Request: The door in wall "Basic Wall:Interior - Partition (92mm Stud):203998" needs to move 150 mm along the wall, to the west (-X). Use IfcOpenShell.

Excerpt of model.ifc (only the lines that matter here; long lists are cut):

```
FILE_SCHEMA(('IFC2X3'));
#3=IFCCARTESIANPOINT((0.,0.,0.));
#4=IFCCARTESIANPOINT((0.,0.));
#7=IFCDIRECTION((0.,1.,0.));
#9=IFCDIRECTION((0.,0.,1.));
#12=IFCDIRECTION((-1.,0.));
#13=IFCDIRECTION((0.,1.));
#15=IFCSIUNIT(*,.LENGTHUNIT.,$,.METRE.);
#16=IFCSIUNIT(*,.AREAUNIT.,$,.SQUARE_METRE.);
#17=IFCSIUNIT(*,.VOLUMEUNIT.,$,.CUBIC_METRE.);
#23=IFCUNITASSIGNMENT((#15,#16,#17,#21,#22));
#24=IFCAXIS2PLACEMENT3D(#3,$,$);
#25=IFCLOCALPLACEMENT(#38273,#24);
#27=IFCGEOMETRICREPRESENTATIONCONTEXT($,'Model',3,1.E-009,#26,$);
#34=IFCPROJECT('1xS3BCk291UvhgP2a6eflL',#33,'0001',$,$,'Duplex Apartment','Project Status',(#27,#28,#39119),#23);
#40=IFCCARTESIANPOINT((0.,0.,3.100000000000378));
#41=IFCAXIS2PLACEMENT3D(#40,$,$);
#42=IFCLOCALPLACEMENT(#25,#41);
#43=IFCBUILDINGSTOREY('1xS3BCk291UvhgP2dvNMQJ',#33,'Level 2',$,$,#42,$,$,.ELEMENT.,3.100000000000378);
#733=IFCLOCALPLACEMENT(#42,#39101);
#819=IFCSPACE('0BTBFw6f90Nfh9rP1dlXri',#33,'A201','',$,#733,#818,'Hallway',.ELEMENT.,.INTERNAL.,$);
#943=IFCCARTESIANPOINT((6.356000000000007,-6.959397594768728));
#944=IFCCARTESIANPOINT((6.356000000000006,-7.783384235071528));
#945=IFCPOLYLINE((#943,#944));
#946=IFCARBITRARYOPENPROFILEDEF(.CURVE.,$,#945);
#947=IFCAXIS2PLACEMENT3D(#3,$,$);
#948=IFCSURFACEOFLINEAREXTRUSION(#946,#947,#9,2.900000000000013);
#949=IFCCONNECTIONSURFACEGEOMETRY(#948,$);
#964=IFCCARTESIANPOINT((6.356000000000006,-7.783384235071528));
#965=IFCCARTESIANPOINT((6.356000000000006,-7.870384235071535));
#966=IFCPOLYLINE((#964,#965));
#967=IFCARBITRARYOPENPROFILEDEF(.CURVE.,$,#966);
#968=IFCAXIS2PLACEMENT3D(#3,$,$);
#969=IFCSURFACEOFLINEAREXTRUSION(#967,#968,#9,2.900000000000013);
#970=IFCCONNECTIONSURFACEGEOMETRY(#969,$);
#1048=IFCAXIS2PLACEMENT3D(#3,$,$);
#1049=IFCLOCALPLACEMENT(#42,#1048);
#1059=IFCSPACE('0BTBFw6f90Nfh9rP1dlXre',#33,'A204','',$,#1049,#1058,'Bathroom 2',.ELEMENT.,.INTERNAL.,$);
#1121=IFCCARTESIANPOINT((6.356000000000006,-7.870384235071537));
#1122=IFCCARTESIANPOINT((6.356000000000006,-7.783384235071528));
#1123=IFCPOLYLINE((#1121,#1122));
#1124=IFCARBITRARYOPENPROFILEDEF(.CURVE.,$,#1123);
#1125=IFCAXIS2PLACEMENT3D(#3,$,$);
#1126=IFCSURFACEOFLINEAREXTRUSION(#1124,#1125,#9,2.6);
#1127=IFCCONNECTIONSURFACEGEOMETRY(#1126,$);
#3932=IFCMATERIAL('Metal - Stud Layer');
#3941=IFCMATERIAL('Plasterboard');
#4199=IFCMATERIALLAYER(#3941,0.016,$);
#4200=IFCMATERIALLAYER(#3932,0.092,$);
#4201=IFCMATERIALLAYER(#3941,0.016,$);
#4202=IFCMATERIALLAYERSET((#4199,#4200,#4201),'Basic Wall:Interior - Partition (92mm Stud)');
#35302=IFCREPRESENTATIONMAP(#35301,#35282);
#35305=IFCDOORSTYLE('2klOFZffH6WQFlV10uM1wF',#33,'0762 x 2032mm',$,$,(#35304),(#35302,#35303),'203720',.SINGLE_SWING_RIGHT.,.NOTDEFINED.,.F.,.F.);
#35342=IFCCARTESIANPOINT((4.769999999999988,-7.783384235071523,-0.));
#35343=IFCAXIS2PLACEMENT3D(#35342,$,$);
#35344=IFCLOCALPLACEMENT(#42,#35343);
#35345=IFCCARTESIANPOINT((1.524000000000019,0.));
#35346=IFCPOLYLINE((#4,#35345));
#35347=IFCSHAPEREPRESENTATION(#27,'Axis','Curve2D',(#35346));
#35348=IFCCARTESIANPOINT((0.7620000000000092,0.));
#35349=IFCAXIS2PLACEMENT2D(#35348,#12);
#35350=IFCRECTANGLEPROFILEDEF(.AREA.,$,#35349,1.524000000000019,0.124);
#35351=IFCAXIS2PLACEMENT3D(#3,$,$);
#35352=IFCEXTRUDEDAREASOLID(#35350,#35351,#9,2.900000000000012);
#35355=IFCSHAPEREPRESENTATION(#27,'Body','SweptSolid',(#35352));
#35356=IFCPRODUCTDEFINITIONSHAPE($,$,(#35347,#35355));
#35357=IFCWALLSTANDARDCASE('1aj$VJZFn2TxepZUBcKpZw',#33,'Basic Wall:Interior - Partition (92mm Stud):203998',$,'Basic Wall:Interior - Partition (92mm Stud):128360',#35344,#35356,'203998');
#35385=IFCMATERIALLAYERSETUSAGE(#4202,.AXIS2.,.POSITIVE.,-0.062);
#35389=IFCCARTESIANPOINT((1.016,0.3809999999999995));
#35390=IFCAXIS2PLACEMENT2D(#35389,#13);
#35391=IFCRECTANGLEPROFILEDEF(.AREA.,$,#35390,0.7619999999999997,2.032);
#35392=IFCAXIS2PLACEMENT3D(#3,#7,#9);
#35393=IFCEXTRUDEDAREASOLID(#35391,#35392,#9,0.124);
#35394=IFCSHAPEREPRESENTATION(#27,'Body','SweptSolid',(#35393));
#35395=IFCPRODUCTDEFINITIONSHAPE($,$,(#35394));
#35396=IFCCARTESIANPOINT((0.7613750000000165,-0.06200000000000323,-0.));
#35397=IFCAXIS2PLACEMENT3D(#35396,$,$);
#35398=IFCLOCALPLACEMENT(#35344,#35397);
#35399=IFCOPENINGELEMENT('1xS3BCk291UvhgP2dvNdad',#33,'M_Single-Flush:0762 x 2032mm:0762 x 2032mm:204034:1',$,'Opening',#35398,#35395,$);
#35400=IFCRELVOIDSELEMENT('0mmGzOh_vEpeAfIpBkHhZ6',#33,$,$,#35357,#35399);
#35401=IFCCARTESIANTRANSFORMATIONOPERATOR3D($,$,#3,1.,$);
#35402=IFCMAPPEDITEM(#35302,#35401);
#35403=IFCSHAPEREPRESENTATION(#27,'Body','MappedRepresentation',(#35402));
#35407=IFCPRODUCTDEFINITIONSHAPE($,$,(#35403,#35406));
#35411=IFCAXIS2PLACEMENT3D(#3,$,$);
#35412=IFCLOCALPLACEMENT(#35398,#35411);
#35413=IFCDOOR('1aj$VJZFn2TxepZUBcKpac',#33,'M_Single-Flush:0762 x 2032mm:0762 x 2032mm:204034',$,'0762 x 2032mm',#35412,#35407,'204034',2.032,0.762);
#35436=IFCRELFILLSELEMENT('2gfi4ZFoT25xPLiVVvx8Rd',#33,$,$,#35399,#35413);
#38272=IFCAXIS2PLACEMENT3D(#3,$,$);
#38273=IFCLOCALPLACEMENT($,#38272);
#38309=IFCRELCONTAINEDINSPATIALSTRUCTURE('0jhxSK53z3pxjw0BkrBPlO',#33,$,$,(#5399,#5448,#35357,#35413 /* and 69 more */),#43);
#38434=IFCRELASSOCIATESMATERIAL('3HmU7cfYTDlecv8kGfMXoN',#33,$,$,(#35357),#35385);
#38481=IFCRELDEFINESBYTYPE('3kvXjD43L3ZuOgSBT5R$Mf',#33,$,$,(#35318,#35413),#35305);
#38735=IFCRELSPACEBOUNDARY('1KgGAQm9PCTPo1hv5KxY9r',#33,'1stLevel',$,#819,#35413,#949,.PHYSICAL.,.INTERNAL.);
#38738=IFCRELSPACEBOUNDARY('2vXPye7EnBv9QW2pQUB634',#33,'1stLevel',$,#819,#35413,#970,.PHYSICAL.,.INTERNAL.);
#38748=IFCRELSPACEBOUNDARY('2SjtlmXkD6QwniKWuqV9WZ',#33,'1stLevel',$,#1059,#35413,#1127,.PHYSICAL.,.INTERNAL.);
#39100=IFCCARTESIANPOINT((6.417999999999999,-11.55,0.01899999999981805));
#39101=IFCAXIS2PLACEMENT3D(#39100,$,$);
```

```python
import numpy as np
import ifcopenshell
import ifcopenshell.api.geometry
import ifcopenshell.util.placement

model = ifcopenshell.open("model.ifc")

door = model.by_guid("1aj$VJZFn2TxepZUBcKpac")
opening = door.FillsVoids[0].RelatingOpeningElement
wall = opening.VoidsElements[0].RelatingBuildingElement

wall_matrix = ifcopenshell.util.placement.get_local_placement(wall.ObjectPlacement)
shift = wall_matrix[:3, 0] * -0.15
before = ifcopenshell.util.placement.get_local_placement(door.ObjectPlacement)[:3, 3].copy()

# The door is placed relative to its opening, so it follows when the opening moves.
matrix = ifcopenshell.util.placement.get_local_placement(opening.ObjectPlacement)
matrix[:3, 3] += shift
ifcopenshell.api.geometry.edit_object_placement(
    model, product=opening, matrix=matrix, is_si=False, should_transform_children=True
)

# Space boundary surfaces are stored in each space's coordinates; move them too.
for rel in door.ProvidesBoundaries:
    if not rel.ConnectionGeometry:
        continue
    surface = rel.ConnectionGeometry.SurfaceOnRelatingElement
    space_matrix = ifcopenshell.util.placement.get_local_placement(rel.RelatingSpace.ObjectPlacement)
    point = np.array(surface.Position.Location.Coordinates) + space_matrix[:3, :3].T @ shift
    surface.Position = model.createIfcAxis2Placement3D(
        model.createIfcCartesianPoint(point.tolist()), surface.Position.Axis, surface.Position.RefDirection
    )

after = ifcopenshell.util.placement.get_local_placement(door.ObjectPlacement)[:3, 3]
print("door moved by", (after - before).round(3) + 0.0)

model.write("model_rev.ifc")
```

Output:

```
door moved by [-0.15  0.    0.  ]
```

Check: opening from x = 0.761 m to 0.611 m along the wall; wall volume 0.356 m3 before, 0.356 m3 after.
